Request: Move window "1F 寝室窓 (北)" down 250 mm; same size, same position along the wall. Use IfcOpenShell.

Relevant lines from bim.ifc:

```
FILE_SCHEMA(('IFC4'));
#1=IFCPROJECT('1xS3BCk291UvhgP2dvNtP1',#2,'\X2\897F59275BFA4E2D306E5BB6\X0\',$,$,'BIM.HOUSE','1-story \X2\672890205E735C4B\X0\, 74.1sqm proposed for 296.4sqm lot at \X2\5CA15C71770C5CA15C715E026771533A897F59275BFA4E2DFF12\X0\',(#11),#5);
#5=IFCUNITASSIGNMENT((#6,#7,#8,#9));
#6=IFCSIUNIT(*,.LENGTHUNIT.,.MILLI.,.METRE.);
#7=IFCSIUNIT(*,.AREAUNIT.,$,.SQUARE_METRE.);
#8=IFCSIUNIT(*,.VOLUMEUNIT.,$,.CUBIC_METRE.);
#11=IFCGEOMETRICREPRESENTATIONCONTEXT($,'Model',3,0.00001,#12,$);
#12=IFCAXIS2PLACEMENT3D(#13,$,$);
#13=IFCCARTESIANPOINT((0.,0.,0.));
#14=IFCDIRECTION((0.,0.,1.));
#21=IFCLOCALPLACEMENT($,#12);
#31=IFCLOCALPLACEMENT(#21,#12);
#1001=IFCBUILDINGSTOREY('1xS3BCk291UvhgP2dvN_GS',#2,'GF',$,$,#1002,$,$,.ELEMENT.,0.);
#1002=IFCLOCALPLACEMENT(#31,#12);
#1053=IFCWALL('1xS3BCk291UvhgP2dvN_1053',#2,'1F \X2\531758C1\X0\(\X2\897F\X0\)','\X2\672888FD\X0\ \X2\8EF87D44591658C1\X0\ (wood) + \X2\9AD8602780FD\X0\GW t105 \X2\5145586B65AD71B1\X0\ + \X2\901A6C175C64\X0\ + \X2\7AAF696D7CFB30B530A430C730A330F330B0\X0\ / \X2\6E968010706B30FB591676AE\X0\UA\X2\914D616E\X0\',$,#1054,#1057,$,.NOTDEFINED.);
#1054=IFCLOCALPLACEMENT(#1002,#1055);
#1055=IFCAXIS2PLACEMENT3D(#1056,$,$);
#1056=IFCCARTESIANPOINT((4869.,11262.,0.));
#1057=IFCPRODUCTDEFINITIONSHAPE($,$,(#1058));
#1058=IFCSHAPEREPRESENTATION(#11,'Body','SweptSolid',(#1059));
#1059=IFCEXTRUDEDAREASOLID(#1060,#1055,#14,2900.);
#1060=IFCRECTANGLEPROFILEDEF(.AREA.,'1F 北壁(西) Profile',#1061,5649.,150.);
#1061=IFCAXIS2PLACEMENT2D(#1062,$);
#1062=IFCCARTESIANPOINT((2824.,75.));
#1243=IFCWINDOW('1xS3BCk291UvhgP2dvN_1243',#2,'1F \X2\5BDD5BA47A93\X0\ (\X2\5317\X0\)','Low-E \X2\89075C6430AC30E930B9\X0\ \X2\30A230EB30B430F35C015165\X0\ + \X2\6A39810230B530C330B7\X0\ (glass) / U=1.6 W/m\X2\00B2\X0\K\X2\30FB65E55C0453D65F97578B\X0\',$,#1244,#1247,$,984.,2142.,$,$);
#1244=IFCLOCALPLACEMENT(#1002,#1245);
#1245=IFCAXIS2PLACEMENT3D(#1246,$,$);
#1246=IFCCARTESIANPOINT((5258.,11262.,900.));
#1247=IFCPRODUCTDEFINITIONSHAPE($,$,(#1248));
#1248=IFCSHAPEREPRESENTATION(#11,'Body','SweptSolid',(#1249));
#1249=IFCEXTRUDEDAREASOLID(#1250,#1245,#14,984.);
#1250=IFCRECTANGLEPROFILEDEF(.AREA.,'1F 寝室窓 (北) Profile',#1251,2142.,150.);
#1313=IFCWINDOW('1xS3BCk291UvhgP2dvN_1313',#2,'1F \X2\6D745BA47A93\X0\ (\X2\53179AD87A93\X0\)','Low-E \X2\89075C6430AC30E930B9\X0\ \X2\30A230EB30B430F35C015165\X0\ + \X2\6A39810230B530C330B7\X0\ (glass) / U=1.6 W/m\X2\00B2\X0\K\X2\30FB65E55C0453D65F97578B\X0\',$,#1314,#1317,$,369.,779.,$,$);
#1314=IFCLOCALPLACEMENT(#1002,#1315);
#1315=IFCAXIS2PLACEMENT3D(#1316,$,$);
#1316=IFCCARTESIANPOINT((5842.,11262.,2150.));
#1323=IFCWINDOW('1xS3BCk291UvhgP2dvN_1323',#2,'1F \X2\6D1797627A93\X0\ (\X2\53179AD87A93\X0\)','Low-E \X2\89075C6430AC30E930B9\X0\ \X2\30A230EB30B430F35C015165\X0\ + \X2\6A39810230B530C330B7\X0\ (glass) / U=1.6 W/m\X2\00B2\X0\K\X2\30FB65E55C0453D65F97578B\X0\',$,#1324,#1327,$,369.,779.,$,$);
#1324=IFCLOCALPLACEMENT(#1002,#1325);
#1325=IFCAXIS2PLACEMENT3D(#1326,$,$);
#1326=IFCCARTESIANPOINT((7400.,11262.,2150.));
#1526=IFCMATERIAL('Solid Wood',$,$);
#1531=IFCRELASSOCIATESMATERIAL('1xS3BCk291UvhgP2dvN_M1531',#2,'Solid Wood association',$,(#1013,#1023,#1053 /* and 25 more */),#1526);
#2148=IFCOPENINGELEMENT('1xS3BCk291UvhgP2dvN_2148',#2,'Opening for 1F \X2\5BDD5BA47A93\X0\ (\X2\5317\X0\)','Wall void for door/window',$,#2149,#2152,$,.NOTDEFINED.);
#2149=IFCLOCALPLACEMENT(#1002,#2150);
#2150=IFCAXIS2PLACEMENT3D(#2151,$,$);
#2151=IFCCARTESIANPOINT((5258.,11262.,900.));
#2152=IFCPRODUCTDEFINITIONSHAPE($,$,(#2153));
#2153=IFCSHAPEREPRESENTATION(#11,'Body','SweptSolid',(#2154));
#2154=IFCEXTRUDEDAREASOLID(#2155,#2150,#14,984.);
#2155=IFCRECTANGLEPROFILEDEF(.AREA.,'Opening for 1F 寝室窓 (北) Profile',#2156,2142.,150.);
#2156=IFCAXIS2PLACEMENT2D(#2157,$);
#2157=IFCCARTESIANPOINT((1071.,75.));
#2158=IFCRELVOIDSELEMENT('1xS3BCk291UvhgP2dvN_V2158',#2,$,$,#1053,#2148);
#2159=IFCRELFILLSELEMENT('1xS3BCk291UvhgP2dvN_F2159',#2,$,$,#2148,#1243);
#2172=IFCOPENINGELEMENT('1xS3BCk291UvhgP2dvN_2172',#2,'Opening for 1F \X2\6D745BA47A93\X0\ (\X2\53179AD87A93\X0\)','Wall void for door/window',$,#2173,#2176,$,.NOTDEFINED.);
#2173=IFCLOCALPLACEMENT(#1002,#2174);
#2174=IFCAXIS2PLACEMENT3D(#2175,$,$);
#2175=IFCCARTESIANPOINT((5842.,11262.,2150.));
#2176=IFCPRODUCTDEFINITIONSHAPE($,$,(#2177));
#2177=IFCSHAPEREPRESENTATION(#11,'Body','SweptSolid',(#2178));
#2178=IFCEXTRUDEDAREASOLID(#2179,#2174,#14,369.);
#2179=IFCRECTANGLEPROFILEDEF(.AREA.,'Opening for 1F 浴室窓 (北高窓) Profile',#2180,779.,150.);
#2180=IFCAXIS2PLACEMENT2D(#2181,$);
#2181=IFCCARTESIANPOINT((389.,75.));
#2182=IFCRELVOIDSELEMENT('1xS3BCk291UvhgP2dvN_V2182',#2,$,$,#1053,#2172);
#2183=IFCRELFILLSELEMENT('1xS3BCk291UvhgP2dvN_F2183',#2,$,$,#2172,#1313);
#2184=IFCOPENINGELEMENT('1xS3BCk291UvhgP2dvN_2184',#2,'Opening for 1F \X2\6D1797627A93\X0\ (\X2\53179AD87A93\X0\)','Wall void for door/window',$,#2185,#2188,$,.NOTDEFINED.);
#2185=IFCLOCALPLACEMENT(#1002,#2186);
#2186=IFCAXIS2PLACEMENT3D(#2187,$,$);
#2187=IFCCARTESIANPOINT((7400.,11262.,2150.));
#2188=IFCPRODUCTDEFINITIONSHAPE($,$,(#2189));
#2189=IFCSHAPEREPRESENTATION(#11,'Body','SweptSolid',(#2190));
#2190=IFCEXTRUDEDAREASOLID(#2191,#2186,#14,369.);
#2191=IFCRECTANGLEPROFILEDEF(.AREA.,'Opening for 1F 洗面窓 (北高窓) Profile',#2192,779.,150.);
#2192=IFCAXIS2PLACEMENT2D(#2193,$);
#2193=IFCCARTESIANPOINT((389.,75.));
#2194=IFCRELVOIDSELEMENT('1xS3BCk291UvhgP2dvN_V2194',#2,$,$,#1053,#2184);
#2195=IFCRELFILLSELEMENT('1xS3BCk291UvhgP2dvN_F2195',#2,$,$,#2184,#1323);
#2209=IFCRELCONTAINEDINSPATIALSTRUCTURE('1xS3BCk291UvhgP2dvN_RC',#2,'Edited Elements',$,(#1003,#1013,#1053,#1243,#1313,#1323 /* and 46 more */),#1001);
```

```python
import numpy as np
import ifcopenshell
import ifcopenshell.api.geometry
import ifcopenshell.util.placement
import ifcopenshell.util.unit

model = ifcopenshell.open("bim.ifc")
unit_scale = ifcopenshell.util.unit.calculate_unit_scale(model)

window = model.by_guid("1xS3BCk291UvhgP2dvN_1243")
opening = window.FillsVoids[0].RelatingOpeningElement
dz = -0.25 / unit_scale

shift = np.array([0.0, 0.0, dz])
# The window is not placed relative to its opening, so move both.
for product in (opening, window):
    matrix = ifcopenshell.util.placement.get_local_placement(product.ObjectPlacement)
    matrix[:3, 3] += shift
    ifcopenshell.api.geometry.edit_object_placement(model, product=product, matrix=matrix, is_si=False)

print(f"moved by {dz * unit_scale:+.3f} m")

model.write("bim_rev.ifc")
```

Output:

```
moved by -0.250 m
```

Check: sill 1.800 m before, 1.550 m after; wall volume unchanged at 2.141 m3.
